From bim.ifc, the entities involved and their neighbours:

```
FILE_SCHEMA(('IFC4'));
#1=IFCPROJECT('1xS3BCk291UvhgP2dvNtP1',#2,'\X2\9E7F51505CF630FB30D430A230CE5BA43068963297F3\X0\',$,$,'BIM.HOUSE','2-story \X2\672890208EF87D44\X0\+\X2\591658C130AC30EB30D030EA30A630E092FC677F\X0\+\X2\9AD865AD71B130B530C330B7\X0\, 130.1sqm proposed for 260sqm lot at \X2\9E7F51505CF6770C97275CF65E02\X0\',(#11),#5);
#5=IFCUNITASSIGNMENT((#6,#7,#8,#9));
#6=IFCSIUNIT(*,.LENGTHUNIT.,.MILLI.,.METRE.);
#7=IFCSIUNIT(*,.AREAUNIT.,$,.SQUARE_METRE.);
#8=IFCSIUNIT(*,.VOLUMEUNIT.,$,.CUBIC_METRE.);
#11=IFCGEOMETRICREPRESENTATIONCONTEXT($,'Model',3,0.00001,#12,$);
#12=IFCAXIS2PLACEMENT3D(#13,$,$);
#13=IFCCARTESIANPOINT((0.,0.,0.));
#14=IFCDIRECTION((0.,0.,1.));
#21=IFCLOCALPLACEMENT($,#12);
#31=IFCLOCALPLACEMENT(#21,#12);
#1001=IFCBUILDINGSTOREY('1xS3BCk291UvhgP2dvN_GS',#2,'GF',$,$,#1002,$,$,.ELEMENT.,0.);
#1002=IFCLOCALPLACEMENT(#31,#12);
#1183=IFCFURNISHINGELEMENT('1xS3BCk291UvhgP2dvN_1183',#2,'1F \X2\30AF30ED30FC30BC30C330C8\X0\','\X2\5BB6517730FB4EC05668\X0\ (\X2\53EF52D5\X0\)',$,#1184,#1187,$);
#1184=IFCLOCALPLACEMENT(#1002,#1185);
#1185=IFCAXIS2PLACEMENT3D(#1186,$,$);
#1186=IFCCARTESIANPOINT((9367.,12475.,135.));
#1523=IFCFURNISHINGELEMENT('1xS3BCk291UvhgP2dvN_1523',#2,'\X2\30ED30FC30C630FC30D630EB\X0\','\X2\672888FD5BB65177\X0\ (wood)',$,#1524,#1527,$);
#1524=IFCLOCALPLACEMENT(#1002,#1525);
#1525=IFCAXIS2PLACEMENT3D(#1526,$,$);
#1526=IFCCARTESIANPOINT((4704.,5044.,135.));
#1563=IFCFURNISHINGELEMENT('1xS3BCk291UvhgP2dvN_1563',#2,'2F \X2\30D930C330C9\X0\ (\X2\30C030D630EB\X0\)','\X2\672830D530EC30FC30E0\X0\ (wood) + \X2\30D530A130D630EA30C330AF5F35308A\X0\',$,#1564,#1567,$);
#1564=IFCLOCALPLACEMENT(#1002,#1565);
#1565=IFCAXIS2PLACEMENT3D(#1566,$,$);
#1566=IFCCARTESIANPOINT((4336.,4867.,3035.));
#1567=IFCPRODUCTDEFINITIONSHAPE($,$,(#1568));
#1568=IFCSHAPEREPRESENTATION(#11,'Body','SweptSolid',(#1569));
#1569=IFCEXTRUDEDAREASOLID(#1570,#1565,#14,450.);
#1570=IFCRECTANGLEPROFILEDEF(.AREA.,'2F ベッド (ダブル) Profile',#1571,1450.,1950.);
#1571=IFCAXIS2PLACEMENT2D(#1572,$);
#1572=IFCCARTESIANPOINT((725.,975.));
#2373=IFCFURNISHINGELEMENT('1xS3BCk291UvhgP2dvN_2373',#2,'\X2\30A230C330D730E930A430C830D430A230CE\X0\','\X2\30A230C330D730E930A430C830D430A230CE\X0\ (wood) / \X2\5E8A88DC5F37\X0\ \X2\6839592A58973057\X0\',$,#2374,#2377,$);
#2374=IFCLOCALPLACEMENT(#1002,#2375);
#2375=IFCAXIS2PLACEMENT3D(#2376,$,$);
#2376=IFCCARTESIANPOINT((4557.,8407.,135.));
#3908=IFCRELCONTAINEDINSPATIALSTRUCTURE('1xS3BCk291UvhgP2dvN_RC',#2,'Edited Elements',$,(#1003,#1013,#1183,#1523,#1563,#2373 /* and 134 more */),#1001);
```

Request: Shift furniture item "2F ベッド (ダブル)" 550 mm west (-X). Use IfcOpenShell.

```python
import ifcopenshell
import ifcopenshell.api.geometry
import ifcopenshell.util.placement

model = ifcopenshell.open("bim.ifc")

item = model.by_guid("1xS3BCk291UvhgP2dvN_1563")
matrix = ifcopenshell.util.placement.get_local_placement(item.ObjectPlacement)
matrix[0, 3] -= 550.0
ifcopenshell.api.geometry.edit_object_placement(model, product=item, matrix=matrix, is_si=False)

print(ifcopenshell.util.placement.get_local_placement(item.ObjectPlacement).round(3) + 0.0)

model.write("bim_rev.ifc")
```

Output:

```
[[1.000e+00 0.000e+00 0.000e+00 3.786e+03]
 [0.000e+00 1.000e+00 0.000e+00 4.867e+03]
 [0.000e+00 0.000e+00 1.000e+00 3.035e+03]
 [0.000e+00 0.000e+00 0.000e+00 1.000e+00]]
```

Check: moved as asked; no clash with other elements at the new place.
